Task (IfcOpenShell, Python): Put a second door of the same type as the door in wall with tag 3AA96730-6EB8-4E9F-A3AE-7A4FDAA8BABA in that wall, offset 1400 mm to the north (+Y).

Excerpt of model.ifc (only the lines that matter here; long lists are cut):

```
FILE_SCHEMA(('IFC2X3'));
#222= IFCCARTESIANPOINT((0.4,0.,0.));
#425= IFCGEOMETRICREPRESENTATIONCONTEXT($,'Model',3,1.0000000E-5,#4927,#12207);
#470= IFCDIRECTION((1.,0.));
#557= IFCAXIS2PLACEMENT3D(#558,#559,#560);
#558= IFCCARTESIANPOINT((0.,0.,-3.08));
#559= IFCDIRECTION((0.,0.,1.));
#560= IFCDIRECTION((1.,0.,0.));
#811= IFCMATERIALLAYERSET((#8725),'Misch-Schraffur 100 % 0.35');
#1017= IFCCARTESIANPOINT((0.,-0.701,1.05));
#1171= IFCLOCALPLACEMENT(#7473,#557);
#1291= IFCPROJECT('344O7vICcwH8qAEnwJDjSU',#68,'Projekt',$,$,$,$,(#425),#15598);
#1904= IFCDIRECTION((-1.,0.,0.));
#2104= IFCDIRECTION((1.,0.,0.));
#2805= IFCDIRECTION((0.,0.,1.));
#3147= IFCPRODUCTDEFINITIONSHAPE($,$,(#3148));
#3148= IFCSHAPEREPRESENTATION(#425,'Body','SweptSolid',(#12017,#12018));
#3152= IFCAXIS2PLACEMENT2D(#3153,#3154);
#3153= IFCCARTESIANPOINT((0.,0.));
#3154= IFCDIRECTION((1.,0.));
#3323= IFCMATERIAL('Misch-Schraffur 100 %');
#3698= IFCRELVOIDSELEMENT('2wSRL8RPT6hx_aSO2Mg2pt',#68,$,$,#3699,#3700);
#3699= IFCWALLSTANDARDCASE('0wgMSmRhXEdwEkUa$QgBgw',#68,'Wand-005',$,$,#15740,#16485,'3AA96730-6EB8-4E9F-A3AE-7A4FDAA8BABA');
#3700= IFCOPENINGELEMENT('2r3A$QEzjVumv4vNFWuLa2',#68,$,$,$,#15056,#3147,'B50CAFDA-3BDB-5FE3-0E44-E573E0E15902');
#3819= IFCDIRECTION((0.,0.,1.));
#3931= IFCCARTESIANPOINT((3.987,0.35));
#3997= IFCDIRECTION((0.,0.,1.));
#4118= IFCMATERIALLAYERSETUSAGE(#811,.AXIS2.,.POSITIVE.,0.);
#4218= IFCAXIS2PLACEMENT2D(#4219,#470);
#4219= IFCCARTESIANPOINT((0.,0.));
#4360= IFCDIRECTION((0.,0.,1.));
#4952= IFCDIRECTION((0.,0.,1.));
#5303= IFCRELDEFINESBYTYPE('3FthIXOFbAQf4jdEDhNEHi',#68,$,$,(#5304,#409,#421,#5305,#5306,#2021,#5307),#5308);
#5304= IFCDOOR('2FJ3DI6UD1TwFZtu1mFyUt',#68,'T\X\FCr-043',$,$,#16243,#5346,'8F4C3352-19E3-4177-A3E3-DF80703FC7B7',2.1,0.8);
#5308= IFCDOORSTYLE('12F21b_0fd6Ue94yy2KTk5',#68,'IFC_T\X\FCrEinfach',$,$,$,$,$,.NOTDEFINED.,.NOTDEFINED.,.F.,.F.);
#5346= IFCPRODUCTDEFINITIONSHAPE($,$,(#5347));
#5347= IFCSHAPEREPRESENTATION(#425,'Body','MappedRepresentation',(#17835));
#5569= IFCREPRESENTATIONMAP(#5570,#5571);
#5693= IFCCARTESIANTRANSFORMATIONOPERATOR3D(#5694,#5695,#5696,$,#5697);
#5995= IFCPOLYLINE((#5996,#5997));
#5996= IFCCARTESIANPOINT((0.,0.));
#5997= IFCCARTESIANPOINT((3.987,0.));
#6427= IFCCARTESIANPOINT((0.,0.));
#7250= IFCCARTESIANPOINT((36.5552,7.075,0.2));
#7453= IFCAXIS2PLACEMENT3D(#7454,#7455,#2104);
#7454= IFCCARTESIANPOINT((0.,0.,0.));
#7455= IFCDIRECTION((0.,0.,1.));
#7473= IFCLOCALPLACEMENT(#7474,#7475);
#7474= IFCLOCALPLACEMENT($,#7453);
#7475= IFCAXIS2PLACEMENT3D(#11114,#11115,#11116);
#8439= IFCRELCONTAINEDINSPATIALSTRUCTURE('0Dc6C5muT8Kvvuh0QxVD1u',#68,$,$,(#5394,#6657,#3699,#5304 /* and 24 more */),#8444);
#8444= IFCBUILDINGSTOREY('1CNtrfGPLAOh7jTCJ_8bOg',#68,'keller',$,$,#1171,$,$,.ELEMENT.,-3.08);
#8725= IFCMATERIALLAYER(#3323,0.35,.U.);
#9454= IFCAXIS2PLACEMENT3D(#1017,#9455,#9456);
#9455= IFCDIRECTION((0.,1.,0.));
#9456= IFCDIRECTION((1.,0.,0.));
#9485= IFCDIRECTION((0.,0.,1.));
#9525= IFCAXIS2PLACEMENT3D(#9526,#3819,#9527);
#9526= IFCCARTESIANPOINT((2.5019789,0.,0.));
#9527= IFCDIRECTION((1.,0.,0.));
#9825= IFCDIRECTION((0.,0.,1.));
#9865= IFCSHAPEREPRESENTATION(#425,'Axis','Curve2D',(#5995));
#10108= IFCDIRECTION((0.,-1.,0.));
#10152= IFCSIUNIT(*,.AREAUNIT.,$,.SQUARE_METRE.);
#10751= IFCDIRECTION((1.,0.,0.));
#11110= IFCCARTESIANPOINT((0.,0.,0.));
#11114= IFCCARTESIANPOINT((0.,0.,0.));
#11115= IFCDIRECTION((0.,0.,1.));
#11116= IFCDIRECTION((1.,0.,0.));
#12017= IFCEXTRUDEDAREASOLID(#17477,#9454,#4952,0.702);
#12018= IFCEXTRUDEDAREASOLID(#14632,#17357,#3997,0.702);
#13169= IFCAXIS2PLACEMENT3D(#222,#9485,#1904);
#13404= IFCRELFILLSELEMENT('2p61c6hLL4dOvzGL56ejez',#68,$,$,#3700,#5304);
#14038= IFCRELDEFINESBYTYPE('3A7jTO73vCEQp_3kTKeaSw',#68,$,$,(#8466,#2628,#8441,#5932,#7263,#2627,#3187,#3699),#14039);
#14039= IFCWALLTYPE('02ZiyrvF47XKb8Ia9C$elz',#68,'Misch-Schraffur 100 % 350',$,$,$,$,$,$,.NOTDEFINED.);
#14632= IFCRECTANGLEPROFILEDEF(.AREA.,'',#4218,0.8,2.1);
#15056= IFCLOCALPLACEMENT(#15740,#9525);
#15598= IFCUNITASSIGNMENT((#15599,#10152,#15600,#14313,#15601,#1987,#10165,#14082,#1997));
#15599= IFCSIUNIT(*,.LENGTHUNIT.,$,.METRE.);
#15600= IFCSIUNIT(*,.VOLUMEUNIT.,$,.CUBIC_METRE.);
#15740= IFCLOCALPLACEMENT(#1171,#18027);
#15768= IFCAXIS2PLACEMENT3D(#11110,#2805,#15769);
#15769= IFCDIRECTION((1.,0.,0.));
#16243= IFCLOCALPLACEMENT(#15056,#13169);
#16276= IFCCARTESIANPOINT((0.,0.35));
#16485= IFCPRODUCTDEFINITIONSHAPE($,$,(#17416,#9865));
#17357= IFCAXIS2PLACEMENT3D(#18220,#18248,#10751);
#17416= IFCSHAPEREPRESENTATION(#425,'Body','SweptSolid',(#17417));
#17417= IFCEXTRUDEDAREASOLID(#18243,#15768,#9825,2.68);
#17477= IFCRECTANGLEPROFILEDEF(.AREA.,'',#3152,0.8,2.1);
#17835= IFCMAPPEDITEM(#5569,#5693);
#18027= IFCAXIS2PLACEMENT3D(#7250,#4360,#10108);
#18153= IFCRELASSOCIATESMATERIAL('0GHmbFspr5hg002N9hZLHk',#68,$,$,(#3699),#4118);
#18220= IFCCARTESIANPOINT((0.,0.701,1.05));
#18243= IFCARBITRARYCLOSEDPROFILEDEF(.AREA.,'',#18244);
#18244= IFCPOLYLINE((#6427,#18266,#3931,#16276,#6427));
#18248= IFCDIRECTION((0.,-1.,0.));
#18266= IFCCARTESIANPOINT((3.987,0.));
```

```python
import ifcopenshell
import ifcopenshell.api.feature
import ifcopenshell.api.geometry
import ifcopenshell.api.root
import ifcopenshell.geom
import ifcopenshell.util.element
import ifcopenshell.util.placement
import ifcopenshell.util.shape
import ifcopenshell.util.unit

model = ifcopenshell.open("model.ifc")
unit_scale = ifcopenshell.util.unit.calculate_unit_scale(model)
settings = ifcopenshell.geom.settings()


def volume(element):
    """Net volume in cubic metres, openings subtracted."""
    shape = ifcopenshell.geom.create_shape(settings, element)
    return ifcopenshell.util.shape.get_volume(shape.geometry)


def reuse_history(source, copy):
    """copy_class also copies each property set's owner history, people and application; keep the originals."""
    for rel in copy.IsDefinedBy:
        if rel.is_a("IfcRelDefinesByProperties") and (history := rel.RelatingPropertyDefinition.OwnerHistory):
            rel.RelatingPropertyDefinition.OwnerHistory = source.OwnerHistory
            ifcopenshell.util.element.remove_deep2(model, history)


door = model.by_guid("2FJ3DI6UD1TwFZtu1mFyUt")
opening = door.FillsVoids[0].RelatingOpeningElement
wall = opening.VoidsElements[0].RelatingBuildingElement
before = volume(wall)
shift = ifcopenshell.util.placement.get_local_placement(wall.ObjectPlacement)[:3, 0] * -1.4 / unit_scale

# copy_class copies the void relationship, type, container and properties, but no geometry.
new_opening = ifcopenshell.api.root.copy_class(model, product=opening)
new_opening.Representation = ifcopenshell.util.element.copy_deep(
    model, opening.Representation, exclude=["IfcGeometricRepresentationContext", "IfcRepresentationMap"]
)
new_opening.Tag = None
new_door = ifcopenshell.api.root.copy_class(model, product=door)
new_door.Representation = ifcopenshell.util.element.copy_deep(
    model, door.Representation, exclude=["IfcGeometricRepresentationContext", "IfcRepresentationMap"]
)
new_door.Tag = None
reuse_history(door, new_door)
fills = ifcopenshell.api.feature.add_filling(model, opening=new_opening, element=new_door)
fills.OwnerHistory = new_door.OwnerHistory  # required in IFC2X3

for old, new in ((opening, new_opening), (door, new_door)):
    matrix = ifcopenshell.util.placement.get_local_placement(old.ObjectPlacement)
    matrix[:3, 3] += shift
    ifcopenshell.api.geometry.edit_object_placement(model, product=new, matrix=matrix, is_si=False)

after = volume(wall)

print(f"wall volume {before:.3f} -> {after:.3f} m3")

model.write("model_v2.ifc")
```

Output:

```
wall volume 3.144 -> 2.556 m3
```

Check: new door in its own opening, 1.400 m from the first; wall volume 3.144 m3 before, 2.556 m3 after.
